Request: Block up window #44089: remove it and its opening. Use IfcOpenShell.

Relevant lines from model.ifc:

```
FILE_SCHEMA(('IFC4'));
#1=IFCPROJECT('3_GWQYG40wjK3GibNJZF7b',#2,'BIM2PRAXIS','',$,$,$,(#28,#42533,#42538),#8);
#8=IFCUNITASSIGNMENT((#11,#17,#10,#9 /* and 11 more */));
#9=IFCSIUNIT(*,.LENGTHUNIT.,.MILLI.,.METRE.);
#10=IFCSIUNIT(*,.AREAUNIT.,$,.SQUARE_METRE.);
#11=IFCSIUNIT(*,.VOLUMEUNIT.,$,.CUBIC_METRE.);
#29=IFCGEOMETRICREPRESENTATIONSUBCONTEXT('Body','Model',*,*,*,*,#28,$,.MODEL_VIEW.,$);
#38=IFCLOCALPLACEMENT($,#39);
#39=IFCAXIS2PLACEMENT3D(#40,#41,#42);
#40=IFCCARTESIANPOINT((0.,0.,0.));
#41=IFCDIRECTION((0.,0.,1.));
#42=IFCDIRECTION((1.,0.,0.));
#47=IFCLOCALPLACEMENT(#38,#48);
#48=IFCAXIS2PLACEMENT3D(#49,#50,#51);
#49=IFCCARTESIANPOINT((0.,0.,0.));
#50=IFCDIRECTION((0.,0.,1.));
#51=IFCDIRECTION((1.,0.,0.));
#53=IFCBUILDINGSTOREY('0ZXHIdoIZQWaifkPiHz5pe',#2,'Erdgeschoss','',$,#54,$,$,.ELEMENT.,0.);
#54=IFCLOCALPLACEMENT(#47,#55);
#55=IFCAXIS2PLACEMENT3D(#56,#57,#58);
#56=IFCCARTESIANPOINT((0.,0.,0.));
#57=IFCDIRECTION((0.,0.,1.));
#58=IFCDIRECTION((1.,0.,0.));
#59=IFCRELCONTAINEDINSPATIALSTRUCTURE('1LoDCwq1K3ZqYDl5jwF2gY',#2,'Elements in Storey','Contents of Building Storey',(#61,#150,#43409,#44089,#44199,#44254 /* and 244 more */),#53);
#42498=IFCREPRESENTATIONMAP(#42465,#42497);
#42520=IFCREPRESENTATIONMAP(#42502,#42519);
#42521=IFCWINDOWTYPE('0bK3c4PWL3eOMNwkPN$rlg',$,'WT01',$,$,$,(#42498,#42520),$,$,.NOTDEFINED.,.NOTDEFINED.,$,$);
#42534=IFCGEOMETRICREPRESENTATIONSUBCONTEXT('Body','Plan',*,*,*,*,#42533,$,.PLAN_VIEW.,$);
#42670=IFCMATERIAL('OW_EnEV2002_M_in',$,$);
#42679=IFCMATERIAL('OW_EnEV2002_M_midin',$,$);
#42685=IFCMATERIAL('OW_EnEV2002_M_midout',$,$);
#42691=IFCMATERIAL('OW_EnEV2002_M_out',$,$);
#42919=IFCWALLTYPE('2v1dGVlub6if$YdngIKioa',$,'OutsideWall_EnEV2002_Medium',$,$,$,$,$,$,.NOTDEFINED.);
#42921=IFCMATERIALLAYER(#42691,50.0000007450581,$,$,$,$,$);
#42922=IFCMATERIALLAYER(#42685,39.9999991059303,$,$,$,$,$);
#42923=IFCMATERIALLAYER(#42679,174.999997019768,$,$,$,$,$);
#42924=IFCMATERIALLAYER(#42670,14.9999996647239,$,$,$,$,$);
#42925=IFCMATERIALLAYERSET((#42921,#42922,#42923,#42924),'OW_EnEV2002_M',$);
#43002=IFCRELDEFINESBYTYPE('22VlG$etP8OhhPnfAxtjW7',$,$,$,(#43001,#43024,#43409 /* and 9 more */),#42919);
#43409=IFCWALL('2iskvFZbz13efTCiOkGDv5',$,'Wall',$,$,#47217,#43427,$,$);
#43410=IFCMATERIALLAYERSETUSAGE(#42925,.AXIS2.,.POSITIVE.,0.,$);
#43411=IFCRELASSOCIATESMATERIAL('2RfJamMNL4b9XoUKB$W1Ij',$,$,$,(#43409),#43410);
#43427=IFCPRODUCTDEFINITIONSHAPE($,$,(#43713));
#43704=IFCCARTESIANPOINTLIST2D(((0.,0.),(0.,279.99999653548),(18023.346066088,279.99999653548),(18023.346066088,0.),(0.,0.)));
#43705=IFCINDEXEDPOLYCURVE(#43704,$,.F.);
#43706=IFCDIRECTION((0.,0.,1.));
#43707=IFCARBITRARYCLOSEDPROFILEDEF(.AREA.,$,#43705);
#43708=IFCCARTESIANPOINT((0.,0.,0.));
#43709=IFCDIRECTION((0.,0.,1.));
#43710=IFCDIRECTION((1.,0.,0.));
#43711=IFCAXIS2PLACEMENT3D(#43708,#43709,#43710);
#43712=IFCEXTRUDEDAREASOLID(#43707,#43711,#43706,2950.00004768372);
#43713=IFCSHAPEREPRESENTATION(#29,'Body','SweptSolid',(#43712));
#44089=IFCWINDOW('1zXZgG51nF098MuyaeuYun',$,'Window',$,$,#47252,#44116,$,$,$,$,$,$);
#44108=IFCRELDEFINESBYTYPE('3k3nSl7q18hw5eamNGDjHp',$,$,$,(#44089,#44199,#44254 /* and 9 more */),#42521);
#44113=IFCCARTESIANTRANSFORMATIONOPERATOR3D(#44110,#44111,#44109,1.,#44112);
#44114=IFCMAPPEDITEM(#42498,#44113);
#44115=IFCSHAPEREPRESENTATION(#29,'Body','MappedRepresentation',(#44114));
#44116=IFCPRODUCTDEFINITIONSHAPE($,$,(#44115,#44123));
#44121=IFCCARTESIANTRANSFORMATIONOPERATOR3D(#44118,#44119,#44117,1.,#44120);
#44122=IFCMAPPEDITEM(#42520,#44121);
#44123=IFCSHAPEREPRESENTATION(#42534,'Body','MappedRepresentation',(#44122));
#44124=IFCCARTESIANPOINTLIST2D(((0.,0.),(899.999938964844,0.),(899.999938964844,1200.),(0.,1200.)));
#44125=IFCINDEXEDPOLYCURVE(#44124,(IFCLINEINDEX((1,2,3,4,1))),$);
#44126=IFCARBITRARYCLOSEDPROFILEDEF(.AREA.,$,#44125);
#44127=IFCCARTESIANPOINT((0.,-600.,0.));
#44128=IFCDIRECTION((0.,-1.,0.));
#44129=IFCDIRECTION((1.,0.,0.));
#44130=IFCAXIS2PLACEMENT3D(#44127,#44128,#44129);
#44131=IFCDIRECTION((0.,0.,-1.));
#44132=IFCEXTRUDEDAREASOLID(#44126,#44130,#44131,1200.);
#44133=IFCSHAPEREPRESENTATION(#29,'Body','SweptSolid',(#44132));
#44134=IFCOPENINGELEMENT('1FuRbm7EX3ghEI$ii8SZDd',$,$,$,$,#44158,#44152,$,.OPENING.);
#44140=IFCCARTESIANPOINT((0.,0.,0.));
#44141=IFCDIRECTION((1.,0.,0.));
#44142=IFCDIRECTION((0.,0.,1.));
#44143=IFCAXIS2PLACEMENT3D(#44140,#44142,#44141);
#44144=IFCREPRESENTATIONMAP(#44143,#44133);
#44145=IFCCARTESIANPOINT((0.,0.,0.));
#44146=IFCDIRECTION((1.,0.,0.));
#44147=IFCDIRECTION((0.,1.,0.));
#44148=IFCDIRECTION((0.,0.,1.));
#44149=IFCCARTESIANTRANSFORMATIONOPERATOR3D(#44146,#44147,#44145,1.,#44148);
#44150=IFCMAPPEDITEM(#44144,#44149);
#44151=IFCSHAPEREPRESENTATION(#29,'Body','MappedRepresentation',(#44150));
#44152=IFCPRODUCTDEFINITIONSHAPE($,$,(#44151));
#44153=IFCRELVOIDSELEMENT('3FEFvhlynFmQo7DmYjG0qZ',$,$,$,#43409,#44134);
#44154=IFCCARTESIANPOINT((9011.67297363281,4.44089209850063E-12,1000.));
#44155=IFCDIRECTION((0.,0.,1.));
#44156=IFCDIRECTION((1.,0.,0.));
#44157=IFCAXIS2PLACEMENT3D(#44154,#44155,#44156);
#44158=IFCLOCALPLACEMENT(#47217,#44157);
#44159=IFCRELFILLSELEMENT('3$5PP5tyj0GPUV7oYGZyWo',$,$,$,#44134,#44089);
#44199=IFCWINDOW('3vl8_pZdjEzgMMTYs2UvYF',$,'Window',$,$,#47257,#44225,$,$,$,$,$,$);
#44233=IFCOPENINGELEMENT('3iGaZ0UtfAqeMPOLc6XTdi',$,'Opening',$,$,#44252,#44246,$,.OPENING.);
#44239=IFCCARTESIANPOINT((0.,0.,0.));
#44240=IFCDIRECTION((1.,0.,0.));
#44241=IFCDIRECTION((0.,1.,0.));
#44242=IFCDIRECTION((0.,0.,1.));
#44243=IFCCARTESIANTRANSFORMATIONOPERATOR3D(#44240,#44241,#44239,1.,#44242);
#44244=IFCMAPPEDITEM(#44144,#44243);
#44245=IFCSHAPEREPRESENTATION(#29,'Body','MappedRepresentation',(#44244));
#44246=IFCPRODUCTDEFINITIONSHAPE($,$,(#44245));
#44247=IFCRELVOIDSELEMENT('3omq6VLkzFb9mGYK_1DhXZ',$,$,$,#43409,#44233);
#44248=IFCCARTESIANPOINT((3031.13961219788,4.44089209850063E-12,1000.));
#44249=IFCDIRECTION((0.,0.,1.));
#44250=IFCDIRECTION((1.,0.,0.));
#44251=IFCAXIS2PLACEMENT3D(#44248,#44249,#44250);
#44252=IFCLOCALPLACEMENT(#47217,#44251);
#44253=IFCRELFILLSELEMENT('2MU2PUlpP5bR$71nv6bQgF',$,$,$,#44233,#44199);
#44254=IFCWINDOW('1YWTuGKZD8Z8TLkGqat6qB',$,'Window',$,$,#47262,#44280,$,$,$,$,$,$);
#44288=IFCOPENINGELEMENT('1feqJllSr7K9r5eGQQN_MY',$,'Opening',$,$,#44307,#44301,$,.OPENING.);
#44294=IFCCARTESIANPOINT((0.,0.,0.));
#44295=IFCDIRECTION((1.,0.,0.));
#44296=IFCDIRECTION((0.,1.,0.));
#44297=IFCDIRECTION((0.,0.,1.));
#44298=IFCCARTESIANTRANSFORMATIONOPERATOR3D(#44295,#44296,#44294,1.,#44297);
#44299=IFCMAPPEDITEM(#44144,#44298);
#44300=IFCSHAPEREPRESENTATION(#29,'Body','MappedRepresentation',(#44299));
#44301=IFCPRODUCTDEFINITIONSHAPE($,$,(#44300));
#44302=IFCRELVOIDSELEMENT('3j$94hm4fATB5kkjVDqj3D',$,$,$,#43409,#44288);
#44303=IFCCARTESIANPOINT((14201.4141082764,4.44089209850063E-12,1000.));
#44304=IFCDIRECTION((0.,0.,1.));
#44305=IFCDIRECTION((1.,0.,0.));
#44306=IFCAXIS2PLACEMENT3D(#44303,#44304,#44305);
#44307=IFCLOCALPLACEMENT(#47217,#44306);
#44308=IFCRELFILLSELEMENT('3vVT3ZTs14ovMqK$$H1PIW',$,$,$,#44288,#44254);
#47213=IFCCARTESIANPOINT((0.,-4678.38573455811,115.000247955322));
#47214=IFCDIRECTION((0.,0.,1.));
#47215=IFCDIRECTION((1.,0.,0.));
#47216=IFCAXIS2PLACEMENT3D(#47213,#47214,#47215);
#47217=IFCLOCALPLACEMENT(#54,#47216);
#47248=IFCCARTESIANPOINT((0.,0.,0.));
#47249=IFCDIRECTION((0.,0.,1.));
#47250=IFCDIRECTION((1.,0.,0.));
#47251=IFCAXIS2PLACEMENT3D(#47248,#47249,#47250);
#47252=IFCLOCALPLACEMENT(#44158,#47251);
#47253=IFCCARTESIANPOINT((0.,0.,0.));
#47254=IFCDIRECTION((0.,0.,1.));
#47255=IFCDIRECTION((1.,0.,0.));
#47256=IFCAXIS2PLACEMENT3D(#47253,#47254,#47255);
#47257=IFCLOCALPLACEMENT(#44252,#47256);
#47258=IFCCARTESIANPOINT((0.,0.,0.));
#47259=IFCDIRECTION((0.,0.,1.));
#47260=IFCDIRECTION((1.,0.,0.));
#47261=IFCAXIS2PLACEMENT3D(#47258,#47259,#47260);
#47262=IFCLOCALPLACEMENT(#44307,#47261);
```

```python
import ifcopenshell
import ifcopenshell.api.feature
import ifcopenshell.api.root
import ifcopenshell.geom
import ifcopenshell.util.shape

model = ifcopenshell.open("model.ifc")
settings = ifcopenshell.geom.settings()


def volume(element):
    """Net volume in cubic metres, openings subtracted."""
    shape = ifcopenshell.geom.create_shape(settings, element)
    return ifcopenshell.util.shape.get_volume(shape.geometry)


window = model.by_guid("1zXZgG51nF098MuyaeuYun")
opening = window.FillsVoids[0].RelatingOpeningElement
wall = opening.VoidsElements[0].RelatingBuildingElement
before = volume(wall)

ifcopenshell.api.root.remove_product(model, product=window)
ifcopenshell.api.feature.remove_feature(model, feature=opening)

after = volume(wall)

print(f"wall volume {before:.3f} -> {after:.3f} m3")

model.write("model-out.ifc")
```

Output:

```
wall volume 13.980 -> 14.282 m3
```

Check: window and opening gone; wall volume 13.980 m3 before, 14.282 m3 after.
